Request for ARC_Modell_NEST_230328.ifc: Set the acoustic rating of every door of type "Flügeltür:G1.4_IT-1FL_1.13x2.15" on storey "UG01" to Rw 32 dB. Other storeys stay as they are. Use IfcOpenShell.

First a look at what the model holds.

```python
import ifcopenshell
import ifcopenshell.util.element

model = ifcopenshell.open("ARC_Modell_NEST_230328.ifc")
print(model.schema)
storey = next(s for s in model.by_type("IfcBuildingStorey") if s.Name == "UG01")
doors = [e for e in ifcopenshell.util.element.get_decomposition(storey) if e.is_a("IfcDoor")]
seen = {}
for e in doors:
    element_type = ifcopenshell.util.element.get_type(e)
    key = (element_type.Name if element_type != e and element_type else None, ifcopenshell.util.element.get_pset(e, "Pset_DoorCommon", "AcousticRating"))
    seen[key] = seen.get(key, 0) + 1
for (name, value), count in sorted(seen.items(), key=str):
    print(count, "x", name, "|", value)
```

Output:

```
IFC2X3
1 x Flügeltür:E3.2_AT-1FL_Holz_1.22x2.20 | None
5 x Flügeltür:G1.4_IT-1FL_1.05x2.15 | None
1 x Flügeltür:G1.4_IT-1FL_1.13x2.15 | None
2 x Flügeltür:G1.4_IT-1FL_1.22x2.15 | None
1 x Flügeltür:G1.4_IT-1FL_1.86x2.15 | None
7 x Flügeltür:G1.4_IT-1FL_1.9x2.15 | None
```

```python
import ifcopenshell
import ifcopenshell.api.pset
import ifcopenshell.util.element

model = ifcopenshell.open("ARC_Modell_NEST_230328.ifc")

storey = next(s for s in model.by_type("IfcBuildingStorey") if s.Name == "UG01")
doors = [e for e in ifcopenshell.util.element.get_decomposition(storey) if e.is_a("IfcDoor")]

count = 0
for e in doors:
    element_type = ifcopenshell.util.element.get_type(e)
    if element_type in (None, e) or element_type.Name != "Flügeltür:G1.4_IT-1FL_1.13x2.15":
        continue
    # add_pset returns the element's existing set when there is one.
    pset = ifcopenshell.api.pset.add_pset(model, product=e, name="Pset_DoorCommon")
    ifcopenshell.api.pset.edit_pset(model, pset=pset, properties={"AcousticRating": "Rw 32 dB"})
    count += 1

print(count, "doors updated")

model.write("ARC_Modell_NEST_230328_updated.ifc")
```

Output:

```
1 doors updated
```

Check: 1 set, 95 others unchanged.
